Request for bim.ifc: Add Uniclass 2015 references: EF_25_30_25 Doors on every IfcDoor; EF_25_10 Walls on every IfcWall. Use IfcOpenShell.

First a look at what the model holds.

```python
import ifcopenshell

model = ifcopenshell.open("bim.ifc")
print(model.schema)
print("classifications:", [c.Name for c in model.by_type("IfcClassification")])
for ifc_class in ("IfcDoor", "IfcRoof", "IfcStair", "IfcWall", "IfcWindow"):
    print(ifc_class, len(model.by_type(ifc_class)))
```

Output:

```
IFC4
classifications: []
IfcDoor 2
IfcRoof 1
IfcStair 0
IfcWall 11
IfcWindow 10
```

```python
import ifcopenshell
import ifcopenshell.api.classification

model = ifcopenshell.open("bim.ifc")

system = ifcopenshell.api.classification.add_classification(model, classification="Uniclass 2015")

codes = {
    "IfcDoor": ("EF_25_30_25", "Doors"),
    "IfcWall": ("EF_25_10", "Walls"),
}
for ifc_class, (code, name) in codes.items():
    products = model.by_type(ifc_class)
    ifcopenshell.api.classification.add_reference(
        model, products=products, classification=system, identification=code, name=name
    )
    print(code, len(products))

model.write("bim_updated.ifc")
```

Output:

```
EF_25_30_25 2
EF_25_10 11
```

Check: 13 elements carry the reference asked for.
